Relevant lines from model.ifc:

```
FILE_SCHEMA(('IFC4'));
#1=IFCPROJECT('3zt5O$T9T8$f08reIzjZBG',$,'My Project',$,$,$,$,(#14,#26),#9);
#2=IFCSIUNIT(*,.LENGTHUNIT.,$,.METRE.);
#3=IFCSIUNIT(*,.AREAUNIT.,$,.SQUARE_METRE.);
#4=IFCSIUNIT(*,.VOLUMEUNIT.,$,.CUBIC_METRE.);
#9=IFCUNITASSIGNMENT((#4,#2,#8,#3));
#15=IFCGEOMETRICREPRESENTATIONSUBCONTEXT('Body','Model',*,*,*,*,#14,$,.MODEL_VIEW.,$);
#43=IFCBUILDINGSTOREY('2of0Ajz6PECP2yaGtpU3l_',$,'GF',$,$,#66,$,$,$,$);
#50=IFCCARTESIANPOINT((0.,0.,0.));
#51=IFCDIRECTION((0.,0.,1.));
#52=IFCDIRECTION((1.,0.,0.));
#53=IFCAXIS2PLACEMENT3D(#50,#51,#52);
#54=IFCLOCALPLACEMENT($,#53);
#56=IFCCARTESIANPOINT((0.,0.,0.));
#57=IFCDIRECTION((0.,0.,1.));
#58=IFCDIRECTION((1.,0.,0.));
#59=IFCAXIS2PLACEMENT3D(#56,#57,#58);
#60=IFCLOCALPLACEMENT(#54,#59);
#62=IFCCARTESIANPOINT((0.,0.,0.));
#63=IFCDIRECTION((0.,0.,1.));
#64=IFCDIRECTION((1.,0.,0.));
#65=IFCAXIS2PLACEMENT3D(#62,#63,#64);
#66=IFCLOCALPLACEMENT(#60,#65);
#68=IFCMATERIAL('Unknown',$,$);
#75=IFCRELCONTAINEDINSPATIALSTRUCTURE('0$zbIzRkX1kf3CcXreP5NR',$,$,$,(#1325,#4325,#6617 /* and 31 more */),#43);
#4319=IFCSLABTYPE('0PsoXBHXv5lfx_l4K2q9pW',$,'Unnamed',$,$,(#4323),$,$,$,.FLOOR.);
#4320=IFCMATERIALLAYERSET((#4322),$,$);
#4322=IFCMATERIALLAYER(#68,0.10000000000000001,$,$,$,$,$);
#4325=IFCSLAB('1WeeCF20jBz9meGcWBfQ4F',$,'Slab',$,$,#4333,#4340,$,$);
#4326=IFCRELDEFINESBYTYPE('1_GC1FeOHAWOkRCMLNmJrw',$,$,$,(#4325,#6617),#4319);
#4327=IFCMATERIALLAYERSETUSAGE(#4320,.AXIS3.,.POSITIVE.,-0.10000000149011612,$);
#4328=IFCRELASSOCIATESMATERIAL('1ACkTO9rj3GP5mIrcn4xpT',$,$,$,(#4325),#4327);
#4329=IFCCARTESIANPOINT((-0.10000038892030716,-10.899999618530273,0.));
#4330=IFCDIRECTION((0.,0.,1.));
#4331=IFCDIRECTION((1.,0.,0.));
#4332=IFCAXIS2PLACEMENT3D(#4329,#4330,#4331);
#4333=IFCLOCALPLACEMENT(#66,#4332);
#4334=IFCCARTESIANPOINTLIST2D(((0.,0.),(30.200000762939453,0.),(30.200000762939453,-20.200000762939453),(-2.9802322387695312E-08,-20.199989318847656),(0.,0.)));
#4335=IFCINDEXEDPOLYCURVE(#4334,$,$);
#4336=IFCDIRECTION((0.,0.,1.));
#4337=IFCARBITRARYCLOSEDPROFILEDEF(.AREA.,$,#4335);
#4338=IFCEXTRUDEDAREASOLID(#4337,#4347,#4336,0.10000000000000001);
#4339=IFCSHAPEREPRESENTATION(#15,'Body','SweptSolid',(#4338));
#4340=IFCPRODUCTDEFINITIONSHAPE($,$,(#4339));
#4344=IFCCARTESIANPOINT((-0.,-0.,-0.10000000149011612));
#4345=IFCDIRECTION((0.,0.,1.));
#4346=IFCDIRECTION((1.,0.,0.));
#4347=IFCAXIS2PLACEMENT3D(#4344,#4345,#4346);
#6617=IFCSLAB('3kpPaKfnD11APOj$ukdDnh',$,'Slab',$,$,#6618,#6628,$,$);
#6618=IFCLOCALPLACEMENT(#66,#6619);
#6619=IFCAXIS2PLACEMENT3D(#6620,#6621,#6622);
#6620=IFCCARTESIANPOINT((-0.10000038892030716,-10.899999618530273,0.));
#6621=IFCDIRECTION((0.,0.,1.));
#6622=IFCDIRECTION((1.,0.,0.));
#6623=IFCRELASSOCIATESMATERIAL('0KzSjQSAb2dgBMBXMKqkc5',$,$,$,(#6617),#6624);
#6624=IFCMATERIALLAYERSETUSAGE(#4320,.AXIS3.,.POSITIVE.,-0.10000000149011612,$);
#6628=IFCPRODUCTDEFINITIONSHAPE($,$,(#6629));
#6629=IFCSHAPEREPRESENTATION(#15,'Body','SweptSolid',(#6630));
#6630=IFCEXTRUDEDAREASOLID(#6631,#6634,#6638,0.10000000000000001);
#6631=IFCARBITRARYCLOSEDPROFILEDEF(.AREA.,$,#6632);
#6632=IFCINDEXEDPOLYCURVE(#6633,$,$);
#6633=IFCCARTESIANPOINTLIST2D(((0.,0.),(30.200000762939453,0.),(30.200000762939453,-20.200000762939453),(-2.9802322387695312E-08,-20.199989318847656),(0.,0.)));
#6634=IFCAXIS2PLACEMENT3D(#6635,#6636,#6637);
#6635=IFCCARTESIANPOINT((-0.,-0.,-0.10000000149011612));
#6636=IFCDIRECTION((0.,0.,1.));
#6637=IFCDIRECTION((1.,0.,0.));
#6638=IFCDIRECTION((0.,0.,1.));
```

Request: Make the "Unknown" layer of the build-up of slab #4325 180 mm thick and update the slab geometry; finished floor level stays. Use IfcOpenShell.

```python
import ifcopenshell
import ifcopenshell.util.element
import ifcopenshell.util.representation

model = ifcopenshell.open("model.ifc")

layer_set = model.by_id(4320)
layer = next(l for l in layer_set.MaterialLayers if l.Material and l.Material.Name == "Unknown")
change = 0.18 - layer.LayerThickness
layer.LayerThickness += change

# The layer set is shared, so every slab that uses it gets the new thickness.
slabs = [e for e in ifcopenshell.util.element.get_elements_by_material(model, layer_set) if e.is_a("IfcSlab")]
for slab in sorted(slabs, key=lambda e: e.id()):
    body = ifcopenshell.util.representation.get_representation(slab, "Model", "Body")
    solid = body.Items[0]
    old_depth = solid.Depth
    solid.Depth += change
    # Extruded upwards: lower the start of the extrusion so the top stays.
    x, y, z = solid.Position.Location.Coordinates
    solid.Position.Location = model.createIfcCartesianPoint((x, y, z - change))
    print(slab.id(), f"{old_depth:g} -> {solid.Depth:g}")

# The layers are counted up from the underside, which has moved.
for usage in {ifcopenshell.util.element.get_material(slab) for slab in slabs}:
    usage.OffsetFromReferenceLine -= change

model.write("model_rev.ifc")
```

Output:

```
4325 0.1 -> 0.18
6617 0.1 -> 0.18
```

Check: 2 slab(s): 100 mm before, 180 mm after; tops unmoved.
